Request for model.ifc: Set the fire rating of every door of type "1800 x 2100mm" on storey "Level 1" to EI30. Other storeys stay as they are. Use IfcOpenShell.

First a look at what the model holds.

```python
import ifcopenshell
import ifcopenshell.util.element

model = ifcopenshell.open("model.ifc")
print(model.schema)
storey = next(s for s in model.by_type("IfcBuildingStorey") if s.Name == "Level 1")
doors = [e for e in ifcopenshell.util.element.get_decomposition(storey) if e.is_a("IfcDoor")]
seen = {}
for e in doors:
    element_type = ifcopenshell.util.element.get_type(e)
    key = (element_type.Name if element_type != e and element_type else None, ifcopenshell.util.element.get_pset(e, "Pset_DoorCommon", "FireRating"))
    seen[key] = seen.get(key, 0) + 1
for (name, value), count in sorted(seen.items(), key=str):
    print(count, "x", name, "|", value)
```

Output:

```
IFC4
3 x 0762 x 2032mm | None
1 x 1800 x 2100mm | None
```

```python
import ifcopenshell
import ifcopenshell.api.pset
import ifcopenshell.util.element

model = ifcopenshell.open("model.ifc")

storey = next(s for s in model.by_type("IfcBuildingStorey") if s.Name == "Level 1")
doors = [e for e in ifcopenshell.util.element.get_decomposition(storey) if e.is_a("IfcDoor")]

count = 0
for e in doors:
    element_type = ifcopenshell.util.element.get_type(e)
    if element_type in (None, e) or element_type.Name != "1800 x 2100mm":
        continue
    # add_pset returns the element's existing set when there is one.
    pset = ifcopenshell.api.pset.add_pset(model, product=e, name="Pset_DoorCommon")
    ifcopenshell.api.pset.edit_pset(model, pset=pset, properties={"FireRating": "EI30"})
    count += 1

print(count, "doors updated")

model.write("model_v2.ifc")
```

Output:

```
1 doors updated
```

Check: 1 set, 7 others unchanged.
